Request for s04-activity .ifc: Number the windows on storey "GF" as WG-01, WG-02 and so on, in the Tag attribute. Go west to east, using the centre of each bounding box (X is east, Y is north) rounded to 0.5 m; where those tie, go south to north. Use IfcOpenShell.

First a look at what the model holds.

```python
import ifcopenshell
import ifcopenshell.util.element
import ifcopenshell.util.placement

model = ifcopenshell.open("s04-activity .ifc")
print(model.schema)
storey = next(s for s in model.by_type("IfcBuildingStorey") if s.Name == "GF")
windows = [e for e in ifcopenshell.util.element.get_decomposition(storey) if e.is_a("IfcWindow")]
for e in sorted(windows, key=lambda e: e.id()):
    origin = ifcopenshell.util.placement.get_local_placement(e.ObjectPlacement)[:3, 3]
    print(e.id(), e.Tag, e.Name, origin.round(2) + 0.0, sep=" | ")
```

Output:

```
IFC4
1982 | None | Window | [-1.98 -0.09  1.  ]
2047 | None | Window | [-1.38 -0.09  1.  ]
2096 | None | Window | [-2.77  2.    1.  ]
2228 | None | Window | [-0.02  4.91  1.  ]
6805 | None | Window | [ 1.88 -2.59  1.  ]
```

```python
import ifcopenshell
import ifcopenshell.geom
import ifcopenshell.util.element
import ifcopenshell.util.shape

model = ifcopenshell.open("s04-activity .ifc")
settings = ifcopenshell.geom.settings()
settings.set("use-world-coords", True)


def centre(element):
    shape = ifcopenshell.geom.create_shape(settings, element)
    return ifcopenshell.util.shape.get_bbox_centroid(shape.geometry)


storey = next(s for s in model.by_type("IfcBuildingStorey") if s.Name == "GF")
windows = [e for e in ifcopenshell.util.element.get_decomposition(storey) if e.is_a("IfcWindow")]

# Insertion points can sit at a corner or the storey origin, so sort by the geometry (in metres).
centres = {e: centre(e) for e in windows}
windows.sort(key=lambda e: (round(centres[e][0] / 0.5), centres[e][1]))

for i, e in enumerate(windows, start=1):
    number = f"WG-{i:02d}"
    e.Tag = number
    print(e.id(), number)

model.write("s04-activity _rev.ifc")
```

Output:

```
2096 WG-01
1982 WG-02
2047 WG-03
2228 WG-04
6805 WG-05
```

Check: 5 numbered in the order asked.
